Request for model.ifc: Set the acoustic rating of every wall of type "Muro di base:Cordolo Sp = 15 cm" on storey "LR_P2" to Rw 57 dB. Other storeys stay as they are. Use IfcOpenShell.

First a look at what the model holds.

```python
import ifcopenshell
import ifcopenshell.util.element

model = ifcopenshell.open("model.ifc")
print(model.schema)
storey = next(s for s in model.by_type("IfcBuildingStorey") if s.Name == "LR_P2")
walls = [e for e in ifcopenshell.util.element.get_decomposition(storey) if e.is_a("IfcWall")]
seen = {}
for e in walls:
    element_type = ifcopenshell.util.element.get_type(e)
    key = (element_type.Name if element_type != e and element_type else None, ifcopenshell.util.element.get_pset(e, "Pset_WallCommon", "AcousticRating"))
    seen[key] = seen.get(key, 0) + 1
for (name, value), count in sorted(seen.items(), key=str):
    print(count, "x", name, "|", value)
```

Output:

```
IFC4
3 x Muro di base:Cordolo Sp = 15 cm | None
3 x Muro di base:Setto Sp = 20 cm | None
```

```python
import ifcopenshell
import ifcopenshell.api.pset
import ifcopenshell.util.element

model = ifcopenshell.open("model.ifc")

storey = next(s for s in model.by_type("IfcBuildingStorey") if s.Name == "LR_P2")
walls = [e for e in ifcopenshell.util.element.get_decomposition(storey) if e.is_a("IfcWall")]

count = 0
for e in walls:
    element_type = ifcopenshell.util.element.get_type(e)
    if element_type in (None, e) or element_type.Name != "Muro di base:Cordolo Sp = 15 cm":
        continue
    # add_pset returns the element's existing set when there is one.
    pset = ifcopenshell.api.pset.add_pset(model, product=e, name="Pset_WallCommon")
    ifcopenshell.api.pset.edit_pset(model, pset=pset, properties={"AcousticRating": "Rw 57 dB"})
    count += 1

print(count, "walls updated")

model.write("model_updated.ifc")
```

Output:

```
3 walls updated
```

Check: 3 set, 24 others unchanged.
